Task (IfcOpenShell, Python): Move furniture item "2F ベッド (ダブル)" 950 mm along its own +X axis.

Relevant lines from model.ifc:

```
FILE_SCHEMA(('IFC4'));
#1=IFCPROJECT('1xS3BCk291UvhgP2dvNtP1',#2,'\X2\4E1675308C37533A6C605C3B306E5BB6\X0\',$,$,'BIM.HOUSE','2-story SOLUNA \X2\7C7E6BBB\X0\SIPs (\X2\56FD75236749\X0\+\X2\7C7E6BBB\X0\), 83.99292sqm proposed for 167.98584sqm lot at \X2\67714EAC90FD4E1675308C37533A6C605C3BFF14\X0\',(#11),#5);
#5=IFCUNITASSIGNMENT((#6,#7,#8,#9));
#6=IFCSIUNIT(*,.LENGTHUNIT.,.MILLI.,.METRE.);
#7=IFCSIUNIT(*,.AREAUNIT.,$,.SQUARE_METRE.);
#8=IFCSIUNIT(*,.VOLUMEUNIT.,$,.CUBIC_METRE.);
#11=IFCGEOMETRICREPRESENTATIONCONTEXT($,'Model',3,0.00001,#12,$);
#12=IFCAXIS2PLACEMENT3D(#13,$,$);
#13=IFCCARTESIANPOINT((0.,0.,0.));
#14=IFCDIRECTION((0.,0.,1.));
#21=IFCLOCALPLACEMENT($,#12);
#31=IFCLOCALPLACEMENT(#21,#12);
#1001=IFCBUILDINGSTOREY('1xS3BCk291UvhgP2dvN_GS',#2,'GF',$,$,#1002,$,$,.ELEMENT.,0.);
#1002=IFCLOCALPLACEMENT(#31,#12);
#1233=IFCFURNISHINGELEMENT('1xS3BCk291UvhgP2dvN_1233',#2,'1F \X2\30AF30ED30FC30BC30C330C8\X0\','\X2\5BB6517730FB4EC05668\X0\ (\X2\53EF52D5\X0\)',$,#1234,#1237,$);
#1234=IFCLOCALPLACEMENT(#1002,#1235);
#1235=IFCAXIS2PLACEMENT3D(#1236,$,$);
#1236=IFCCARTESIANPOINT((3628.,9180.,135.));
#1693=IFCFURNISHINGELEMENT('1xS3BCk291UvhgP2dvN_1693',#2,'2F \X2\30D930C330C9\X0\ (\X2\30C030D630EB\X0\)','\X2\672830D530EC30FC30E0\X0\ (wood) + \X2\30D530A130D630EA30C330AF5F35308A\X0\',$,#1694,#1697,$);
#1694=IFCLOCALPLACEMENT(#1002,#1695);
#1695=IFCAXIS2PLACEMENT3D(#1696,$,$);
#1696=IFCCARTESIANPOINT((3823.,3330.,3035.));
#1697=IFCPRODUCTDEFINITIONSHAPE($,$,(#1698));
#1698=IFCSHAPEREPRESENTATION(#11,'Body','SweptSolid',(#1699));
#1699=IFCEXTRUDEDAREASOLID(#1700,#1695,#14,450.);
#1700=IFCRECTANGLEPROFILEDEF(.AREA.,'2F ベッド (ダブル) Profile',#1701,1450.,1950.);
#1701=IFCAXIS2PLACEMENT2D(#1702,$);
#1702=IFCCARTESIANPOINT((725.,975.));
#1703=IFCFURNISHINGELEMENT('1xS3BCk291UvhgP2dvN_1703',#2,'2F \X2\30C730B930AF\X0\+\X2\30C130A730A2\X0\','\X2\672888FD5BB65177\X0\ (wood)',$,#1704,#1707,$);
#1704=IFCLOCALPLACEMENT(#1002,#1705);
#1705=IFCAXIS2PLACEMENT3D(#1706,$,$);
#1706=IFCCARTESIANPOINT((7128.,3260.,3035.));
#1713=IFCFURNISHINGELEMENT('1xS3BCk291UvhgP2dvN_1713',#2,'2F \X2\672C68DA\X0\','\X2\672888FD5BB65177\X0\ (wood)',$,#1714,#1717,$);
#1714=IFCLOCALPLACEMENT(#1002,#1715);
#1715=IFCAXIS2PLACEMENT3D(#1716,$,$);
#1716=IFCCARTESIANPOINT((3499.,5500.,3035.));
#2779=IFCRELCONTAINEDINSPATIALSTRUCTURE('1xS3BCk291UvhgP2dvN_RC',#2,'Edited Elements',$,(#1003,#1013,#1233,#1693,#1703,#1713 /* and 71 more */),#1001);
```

```python
import ifcopenshell
import ifcopenshell.api.geometry
import ifcopenshell.util.placement
import ifcopenshell.util.unit

model = ifcopenshell.open("model.ifc")
unit_scale = ifcopenshell.util.unit.calculate_unit_scale(model)

item = model.by_guid("1xS3BCk291UvhgP2dvN_1693")
matrix = ifcopenshell.util.placement.get_local_placement(item.ObjectPlacement)
matrix[:3, 3] += matrix[:3, 0] * 0.95 / unit_scale
ifcopenshell.api.geometry.edit_object_placement(model, product=item, matrix=matrix, is_si=False)

print(ifcopenshell.util.placement.get_local_placement(item.ObjectPlacement).round(3) + 0.0)

model.write("model_rev.ifc")
```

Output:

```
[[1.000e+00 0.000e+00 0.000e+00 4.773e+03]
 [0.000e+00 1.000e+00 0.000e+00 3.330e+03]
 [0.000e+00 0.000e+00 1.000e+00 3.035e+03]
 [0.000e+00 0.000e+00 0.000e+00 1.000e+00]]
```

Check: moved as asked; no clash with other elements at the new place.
